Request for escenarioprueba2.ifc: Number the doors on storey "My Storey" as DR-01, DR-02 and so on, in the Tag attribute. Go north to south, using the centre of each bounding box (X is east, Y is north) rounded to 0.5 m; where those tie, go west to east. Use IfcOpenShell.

First a look at what the model holds.

```python
import ifcopenshell
import ifcopenshell.util.element
import ifcopenshell.util.placement

model = ifcopenshell.open("escenarioprueba2.ifc")
print(model.schema)
storey = next(s for s in model.by_type("IfcBuildingStorey") if s.Name == "My Storey")
doors = [e for e in ifcopenshell.util.element.get_decomposition(storey) if e.is_a("IfcDoor")]
for e in sorted(doors, key=lambda e: e.id()):
    origin = ifcopenshell.util.placement.get_local_placement(e.ObjectPlacement)[:3, 3]
    print(e.id(), e.Tag, e.Name, origin.round(2) + 0.0, sep=" | ")
```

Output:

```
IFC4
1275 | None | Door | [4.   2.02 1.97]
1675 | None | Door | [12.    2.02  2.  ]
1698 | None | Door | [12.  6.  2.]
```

```python
import ifcopenshell
import ifcopenshell.geom
import ifcopenshell.util.element
import ifcopenshell.util.shape

model = ifcopenshell.open("escenarioprueba2.ifc")
settings = ifcopenshell.geom.settings()
settings.set("use-world-coords", True)


def centre(element):
    shape = ifcopenshell.geom.create_shape(settings, element)
    return ifcopenshell.util.shape.get_bbox_centroid(shape.geometry)


storey = next(s for s in model.by_type("IfcBuildingStorey") if s.Name == "My Storey")
doors = [e for e in ifcopenshell.util.element.get_decomposition(storey) if e.is_a("IfcDoor")]

# Insertion points can sit at a corner or the storey origin, so sort by the geometry (in metres).
centres = {e: centre(e) for e in doors}
doors.sort(key=lambda e: (-round(centres[e][1] / 0.5), centres[e][0]))

for i, e in enumerate(doors, start=1):
    number = f"DR-{i:02d}"
    e.Tag = number
    print(e.id(), number)

model.write("escenarioprueba2_rev.ifc")
```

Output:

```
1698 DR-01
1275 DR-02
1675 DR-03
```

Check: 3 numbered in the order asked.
